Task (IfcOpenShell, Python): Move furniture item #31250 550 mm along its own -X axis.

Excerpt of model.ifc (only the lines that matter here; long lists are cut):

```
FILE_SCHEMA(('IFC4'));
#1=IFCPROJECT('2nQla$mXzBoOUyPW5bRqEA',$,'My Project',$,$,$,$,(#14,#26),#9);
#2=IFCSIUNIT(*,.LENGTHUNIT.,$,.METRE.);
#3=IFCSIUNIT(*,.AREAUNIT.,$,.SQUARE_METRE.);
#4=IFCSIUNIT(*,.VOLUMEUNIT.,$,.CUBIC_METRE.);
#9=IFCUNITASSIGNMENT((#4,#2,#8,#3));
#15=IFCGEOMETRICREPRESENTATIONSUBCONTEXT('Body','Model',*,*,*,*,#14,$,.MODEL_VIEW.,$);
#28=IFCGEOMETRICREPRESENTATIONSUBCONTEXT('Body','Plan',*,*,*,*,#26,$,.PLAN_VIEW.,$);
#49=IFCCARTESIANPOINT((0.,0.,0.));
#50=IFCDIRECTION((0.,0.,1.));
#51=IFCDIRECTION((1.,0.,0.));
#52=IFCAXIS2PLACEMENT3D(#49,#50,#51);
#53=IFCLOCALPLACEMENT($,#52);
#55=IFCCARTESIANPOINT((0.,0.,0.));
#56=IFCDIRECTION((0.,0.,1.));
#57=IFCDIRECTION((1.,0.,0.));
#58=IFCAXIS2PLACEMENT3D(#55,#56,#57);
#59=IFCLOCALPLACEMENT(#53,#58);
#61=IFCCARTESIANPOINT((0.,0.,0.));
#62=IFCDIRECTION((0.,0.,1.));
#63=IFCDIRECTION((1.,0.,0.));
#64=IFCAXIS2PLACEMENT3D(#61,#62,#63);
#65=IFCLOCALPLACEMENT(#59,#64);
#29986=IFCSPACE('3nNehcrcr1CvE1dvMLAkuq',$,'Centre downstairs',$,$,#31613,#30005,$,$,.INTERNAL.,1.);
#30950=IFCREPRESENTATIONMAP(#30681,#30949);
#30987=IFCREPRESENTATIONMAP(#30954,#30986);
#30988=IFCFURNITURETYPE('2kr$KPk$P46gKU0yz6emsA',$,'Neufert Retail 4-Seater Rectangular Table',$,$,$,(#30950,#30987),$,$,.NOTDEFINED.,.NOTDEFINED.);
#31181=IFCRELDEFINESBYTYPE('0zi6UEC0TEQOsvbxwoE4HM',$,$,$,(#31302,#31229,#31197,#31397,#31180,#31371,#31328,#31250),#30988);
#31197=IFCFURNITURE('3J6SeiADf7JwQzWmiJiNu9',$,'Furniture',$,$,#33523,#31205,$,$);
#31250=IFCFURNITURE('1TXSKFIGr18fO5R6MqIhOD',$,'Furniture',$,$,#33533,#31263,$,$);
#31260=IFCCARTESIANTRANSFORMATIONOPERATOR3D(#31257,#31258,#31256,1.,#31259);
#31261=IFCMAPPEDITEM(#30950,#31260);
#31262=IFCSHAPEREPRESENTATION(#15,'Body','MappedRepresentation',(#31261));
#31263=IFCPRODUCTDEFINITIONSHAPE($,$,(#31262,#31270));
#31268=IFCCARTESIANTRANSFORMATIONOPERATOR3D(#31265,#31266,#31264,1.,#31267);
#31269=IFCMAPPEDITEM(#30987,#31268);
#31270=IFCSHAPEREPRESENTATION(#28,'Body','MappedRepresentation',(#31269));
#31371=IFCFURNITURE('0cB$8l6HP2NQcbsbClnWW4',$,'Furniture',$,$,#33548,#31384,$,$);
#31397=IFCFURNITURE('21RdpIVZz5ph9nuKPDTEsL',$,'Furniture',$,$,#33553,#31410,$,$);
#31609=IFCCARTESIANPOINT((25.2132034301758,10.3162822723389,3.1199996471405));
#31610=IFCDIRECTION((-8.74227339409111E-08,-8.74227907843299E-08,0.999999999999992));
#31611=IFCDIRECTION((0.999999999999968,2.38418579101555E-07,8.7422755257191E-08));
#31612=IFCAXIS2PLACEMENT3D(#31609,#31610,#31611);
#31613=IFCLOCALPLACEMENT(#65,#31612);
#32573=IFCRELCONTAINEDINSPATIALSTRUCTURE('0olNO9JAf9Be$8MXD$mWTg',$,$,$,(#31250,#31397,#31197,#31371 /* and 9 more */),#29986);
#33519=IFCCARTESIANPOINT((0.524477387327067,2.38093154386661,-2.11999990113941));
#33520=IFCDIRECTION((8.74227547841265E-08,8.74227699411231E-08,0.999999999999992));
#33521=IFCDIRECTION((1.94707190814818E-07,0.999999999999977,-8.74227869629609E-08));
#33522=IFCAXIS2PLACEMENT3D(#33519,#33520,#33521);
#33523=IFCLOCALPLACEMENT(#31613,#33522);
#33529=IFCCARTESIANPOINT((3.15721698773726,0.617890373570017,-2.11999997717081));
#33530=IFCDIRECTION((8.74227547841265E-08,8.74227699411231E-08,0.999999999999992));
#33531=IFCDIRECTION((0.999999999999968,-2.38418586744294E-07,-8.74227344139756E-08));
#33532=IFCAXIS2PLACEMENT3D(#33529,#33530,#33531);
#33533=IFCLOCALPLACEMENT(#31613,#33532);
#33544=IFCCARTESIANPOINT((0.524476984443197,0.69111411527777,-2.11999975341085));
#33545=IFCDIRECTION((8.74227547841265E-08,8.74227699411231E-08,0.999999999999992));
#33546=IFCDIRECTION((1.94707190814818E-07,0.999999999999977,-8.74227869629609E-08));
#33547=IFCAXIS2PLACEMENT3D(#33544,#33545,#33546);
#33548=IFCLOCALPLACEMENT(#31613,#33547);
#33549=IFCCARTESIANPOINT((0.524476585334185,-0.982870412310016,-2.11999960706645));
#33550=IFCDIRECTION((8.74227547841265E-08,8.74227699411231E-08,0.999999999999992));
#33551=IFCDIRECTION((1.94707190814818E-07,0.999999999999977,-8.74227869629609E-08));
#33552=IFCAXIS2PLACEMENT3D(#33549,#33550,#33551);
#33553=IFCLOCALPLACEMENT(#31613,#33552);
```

```python
import ifcopenshell
import ifcopenshell.api.geometry
import ifcopenshell.util.placement
import ifcopenshell.util.unit

model = ifcopenshell.open("model.ifc")
unit_scale = ifcopenshell.util.unit.calculate_unit_scale(model)

item = model.by_guid("1TXSKFIGr18fO5R6MqIhOD")
matrix = ifcopenshell.util.placement.get_local_placement(item.ObjectPlacement)
matrix[:3, 3] -= matrix[:3, 0] * 0.55 / unit_scale
ifcopenshell.api.geometry.edit_object_placement(model, product=item, matrix=matrix, is_si=False)

print(ifcopenshell.util.placement.get_local_placement(item.ObjectPlacement).round(3) + 0.0)

model.write("model_updated.ifc")
```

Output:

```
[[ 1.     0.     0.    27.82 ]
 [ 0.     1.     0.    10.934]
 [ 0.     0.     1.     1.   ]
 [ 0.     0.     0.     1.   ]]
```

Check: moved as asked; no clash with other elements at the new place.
